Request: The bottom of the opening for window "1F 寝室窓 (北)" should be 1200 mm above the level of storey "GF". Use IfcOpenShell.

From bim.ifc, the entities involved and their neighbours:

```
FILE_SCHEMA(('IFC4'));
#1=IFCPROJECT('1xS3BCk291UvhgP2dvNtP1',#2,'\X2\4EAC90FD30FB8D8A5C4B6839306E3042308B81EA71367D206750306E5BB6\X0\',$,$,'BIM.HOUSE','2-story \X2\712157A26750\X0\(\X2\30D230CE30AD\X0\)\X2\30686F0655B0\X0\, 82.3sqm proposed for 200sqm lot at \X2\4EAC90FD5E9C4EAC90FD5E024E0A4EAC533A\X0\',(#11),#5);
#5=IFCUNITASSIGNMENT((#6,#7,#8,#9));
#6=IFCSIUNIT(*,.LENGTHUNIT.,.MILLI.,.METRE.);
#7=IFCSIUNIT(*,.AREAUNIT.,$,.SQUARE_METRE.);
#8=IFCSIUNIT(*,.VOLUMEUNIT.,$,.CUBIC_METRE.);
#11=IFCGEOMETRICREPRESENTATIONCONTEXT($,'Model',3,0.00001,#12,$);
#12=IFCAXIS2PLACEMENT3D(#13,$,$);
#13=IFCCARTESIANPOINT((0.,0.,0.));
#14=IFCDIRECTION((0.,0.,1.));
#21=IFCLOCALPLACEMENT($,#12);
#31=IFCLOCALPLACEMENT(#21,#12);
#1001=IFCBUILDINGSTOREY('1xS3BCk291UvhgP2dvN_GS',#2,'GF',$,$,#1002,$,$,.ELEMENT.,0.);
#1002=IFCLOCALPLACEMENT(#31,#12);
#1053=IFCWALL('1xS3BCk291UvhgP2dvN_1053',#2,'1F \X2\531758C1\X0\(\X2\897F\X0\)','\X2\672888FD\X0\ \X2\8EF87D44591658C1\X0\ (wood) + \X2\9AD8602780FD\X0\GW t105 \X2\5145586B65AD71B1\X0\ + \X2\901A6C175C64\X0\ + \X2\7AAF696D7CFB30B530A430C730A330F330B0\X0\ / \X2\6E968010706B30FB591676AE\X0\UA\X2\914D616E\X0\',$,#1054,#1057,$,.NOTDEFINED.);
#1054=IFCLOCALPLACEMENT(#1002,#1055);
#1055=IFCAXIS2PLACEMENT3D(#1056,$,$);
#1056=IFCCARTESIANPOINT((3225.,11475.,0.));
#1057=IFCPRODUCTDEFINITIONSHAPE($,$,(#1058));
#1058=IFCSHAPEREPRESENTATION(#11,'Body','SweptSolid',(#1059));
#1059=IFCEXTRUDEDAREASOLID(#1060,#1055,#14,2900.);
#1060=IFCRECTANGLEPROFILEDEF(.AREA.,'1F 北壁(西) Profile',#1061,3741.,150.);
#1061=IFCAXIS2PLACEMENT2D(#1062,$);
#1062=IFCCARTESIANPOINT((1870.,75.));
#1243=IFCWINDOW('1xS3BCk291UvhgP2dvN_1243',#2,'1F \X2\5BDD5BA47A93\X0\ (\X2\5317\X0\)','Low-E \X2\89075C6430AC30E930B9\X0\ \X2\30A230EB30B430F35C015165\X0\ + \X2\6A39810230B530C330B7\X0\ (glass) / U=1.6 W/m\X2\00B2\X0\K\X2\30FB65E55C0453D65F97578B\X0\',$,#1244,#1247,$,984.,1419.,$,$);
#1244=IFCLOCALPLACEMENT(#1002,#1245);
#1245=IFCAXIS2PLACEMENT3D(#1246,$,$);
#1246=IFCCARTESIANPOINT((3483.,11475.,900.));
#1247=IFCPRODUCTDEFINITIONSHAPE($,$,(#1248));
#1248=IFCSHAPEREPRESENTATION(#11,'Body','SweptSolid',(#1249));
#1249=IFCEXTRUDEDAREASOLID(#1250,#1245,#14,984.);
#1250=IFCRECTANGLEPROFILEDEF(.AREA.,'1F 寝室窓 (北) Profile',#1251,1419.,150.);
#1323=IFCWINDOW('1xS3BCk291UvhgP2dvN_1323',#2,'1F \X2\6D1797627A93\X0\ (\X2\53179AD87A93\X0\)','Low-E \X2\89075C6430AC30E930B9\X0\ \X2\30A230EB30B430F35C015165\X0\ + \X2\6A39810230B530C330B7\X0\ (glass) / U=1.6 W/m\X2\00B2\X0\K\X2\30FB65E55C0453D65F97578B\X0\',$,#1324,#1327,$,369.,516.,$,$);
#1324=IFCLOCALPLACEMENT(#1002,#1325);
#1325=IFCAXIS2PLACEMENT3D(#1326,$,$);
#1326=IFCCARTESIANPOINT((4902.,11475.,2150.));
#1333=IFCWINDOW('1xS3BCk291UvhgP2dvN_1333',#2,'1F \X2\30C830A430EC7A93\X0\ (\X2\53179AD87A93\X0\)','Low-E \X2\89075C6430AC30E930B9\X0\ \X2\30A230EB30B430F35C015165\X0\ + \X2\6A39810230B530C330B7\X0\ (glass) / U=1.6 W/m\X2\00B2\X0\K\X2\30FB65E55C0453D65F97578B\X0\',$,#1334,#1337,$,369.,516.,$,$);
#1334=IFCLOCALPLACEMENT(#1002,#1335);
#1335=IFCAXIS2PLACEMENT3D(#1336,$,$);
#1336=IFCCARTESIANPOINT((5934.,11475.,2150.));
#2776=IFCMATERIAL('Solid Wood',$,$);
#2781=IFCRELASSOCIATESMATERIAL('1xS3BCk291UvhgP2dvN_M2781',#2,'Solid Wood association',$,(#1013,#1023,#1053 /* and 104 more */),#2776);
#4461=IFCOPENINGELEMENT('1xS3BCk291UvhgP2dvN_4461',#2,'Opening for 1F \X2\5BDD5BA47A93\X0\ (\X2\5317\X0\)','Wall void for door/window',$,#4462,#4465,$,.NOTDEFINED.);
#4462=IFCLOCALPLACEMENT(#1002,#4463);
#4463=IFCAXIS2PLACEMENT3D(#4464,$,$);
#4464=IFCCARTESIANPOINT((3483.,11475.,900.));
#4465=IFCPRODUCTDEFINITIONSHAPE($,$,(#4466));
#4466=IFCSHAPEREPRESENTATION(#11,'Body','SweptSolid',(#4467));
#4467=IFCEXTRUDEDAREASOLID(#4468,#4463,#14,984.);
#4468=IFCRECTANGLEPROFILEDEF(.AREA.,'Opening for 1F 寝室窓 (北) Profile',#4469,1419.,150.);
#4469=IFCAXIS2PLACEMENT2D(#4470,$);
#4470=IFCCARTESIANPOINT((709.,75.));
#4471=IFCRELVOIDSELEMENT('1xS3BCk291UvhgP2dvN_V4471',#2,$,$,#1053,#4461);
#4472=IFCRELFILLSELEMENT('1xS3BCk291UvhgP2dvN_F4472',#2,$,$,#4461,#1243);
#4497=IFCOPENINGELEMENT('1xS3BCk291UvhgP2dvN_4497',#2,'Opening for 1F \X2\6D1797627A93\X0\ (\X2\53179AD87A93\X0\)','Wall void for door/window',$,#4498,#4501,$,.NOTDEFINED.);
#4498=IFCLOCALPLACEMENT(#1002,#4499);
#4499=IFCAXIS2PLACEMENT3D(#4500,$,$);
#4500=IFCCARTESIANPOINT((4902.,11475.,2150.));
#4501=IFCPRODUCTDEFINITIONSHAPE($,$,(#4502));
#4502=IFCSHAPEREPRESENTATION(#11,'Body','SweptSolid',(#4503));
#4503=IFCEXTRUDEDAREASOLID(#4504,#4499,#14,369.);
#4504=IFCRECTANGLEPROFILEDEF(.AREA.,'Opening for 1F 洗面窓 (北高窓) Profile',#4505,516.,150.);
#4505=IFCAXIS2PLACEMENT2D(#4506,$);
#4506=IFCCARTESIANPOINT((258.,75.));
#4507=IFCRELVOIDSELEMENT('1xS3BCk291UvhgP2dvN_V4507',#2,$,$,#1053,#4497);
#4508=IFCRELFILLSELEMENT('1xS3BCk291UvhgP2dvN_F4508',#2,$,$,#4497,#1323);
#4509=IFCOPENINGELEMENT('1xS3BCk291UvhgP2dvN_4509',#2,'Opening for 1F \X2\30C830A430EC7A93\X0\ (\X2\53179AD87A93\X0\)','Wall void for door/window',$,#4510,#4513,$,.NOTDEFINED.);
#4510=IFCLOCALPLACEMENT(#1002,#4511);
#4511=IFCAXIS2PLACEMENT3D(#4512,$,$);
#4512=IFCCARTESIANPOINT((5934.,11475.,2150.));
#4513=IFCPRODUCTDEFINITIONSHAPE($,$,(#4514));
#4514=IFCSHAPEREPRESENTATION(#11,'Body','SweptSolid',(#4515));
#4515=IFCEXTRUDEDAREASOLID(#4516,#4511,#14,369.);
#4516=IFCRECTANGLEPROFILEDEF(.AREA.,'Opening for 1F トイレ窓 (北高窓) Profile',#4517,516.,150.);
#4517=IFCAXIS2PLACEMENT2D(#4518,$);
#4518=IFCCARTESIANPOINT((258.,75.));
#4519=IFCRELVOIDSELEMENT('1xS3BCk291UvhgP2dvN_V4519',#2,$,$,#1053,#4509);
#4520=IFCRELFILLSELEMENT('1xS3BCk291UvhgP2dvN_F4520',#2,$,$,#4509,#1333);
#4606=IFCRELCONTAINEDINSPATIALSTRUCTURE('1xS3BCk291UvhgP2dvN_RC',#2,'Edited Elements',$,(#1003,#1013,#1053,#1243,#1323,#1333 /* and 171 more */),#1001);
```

```python
import numpy as np
import ifcopenshell
import ifcopenshell.api.geometry
import ifcopenshell.geom
import ifcopenshell.util.element
import ifcopenshell.util.placement
import ifcopenshell.util.shape
import ifcopenshell.util.unit

model = ifcopenshell.open("bim.ifc")
unit_scale = ifcopenshell.util.unit.calculate_unit_scale(model)

window = model.by_guid("1xS3BCk291UvhgP2dvN_1243")
opening = window.FillsVoids[0].RelatingOpeningElement
storey = ifcopenshell.util.element.get_container(window, ifc_class="IfcBuildingStorey")
level = ifcopenshell.util.placement.get_local_placement(storey.ObjectPlacement)[2, 3]

# The opening's origin need not be at the sill, so measure its lowest point.
shape = ifcopenshell.geom.create_shape(ifcopenshell.geom.settings(), opening)
bottom = ifcopenshell.util.shape.get_shape_bottom_elevation(shape, shape.geometry) / unit_scale
dz = level + 1.2 / unit_scale - bottom

shift = np.array([0.0, 0.0, dz])
# The window is not placed relative to its opening, so move both.
for product in (opening, window):
    matrix = ifcopenshell.util.placement.get_local_placement(product.ObjectPlacement)
    matrix[:3, 3] += shift
    ifcopenshell.api.geometry.edit_object_placement(model, product=product, matrix=matrix, is_si=False)

print(f"moved by {dz * unit_scale:+.3f} m")

model.write("bim_rev.ifc")
```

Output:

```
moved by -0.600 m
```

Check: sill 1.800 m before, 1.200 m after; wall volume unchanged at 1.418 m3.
